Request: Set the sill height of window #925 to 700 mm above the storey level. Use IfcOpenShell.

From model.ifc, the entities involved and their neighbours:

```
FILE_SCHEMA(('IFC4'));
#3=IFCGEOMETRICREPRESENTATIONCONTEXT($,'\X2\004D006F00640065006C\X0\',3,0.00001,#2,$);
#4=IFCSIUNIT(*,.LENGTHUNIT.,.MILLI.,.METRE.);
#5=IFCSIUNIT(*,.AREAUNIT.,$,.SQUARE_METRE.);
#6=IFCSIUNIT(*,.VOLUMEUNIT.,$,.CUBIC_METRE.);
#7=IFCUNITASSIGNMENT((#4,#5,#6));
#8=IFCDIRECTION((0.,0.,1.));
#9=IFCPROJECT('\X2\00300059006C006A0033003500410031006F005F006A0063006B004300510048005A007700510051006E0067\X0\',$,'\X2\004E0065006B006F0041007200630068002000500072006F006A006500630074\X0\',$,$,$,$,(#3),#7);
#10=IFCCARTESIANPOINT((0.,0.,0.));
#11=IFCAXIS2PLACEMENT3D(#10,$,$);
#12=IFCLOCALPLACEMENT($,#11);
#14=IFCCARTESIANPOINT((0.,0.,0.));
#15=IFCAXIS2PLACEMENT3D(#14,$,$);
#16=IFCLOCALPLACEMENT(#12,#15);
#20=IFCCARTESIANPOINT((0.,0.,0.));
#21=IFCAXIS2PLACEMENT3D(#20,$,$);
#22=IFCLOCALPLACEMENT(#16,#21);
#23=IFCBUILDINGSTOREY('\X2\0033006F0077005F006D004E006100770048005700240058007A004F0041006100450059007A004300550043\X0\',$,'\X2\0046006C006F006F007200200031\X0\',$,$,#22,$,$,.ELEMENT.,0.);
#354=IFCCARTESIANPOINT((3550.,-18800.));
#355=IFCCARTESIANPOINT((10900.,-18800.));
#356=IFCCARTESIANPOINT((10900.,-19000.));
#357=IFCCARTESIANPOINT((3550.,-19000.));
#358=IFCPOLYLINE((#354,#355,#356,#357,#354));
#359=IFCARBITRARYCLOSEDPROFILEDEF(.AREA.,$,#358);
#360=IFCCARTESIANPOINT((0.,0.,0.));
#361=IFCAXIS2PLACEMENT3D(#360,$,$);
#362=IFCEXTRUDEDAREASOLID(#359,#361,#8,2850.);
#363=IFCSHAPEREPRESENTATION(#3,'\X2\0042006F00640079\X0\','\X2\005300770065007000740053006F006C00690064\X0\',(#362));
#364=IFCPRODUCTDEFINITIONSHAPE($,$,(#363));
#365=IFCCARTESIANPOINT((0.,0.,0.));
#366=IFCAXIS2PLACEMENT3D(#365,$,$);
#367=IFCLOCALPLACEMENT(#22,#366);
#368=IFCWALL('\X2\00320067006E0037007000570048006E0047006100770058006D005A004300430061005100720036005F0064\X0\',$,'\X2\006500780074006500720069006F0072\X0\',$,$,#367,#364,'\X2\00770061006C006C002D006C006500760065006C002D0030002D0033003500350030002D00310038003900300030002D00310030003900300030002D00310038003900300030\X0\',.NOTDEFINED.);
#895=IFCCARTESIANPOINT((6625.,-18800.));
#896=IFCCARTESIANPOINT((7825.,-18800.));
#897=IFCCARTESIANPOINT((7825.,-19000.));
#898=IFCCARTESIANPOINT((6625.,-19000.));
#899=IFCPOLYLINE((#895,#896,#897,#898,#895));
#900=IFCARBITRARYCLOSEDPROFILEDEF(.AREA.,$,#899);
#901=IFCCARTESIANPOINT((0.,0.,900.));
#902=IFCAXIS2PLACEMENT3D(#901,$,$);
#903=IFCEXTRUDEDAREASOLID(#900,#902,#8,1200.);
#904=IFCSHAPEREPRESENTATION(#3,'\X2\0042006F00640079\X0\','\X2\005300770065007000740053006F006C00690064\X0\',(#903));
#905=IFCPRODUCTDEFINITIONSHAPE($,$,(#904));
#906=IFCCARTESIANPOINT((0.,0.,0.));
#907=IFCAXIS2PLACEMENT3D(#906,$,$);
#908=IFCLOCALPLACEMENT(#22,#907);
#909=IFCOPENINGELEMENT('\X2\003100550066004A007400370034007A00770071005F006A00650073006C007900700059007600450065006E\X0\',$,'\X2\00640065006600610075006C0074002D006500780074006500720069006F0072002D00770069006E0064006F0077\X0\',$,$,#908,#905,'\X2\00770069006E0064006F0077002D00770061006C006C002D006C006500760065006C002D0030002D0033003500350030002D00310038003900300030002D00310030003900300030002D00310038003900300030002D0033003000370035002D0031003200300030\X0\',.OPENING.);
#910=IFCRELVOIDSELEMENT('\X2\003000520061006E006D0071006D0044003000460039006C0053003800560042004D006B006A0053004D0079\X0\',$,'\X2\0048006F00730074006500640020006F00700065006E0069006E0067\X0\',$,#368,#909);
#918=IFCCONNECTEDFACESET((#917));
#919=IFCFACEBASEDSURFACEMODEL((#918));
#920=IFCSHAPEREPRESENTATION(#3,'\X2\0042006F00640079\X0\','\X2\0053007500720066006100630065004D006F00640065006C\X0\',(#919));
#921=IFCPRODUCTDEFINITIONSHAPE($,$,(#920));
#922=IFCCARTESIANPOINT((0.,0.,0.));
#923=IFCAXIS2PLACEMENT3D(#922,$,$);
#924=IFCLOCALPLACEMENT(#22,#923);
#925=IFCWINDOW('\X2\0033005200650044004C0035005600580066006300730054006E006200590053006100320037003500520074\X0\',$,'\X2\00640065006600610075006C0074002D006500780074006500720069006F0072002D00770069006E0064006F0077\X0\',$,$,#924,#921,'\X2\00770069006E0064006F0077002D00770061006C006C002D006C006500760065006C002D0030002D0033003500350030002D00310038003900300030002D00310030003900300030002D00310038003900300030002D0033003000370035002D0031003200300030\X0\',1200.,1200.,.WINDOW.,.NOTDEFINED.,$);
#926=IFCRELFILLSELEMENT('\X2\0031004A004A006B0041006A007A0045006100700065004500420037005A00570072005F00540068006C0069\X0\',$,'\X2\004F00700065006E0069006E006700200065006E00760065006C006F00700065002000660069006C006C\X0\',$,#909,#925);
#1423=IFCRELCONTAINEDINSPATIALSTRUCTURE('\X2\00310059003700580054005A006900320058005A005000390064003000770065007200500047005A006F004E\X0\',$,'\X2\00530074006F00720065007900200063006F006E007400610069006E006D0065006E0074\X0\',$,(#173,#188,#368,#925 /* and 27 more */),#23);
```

```python
import numpy as np
import ifcopenshell
import ifcopenshell.api.geometry
import ifcopenshell.geom
import ifcopenshell.util.element
import ifcopenshell.util.placement
import ifcopenshell.util.shape
import ifcopenshell.util.unit

model = ifcopenshell.open("model.ifc")
unit_scale = ifcopenshell.util.unit.calculate_unit_scale(model)

window = model.by_guid("3ReDL5VXfcsTnbYSa275Rt")
opening = window.FillsVoids[0].RelatingOpeningElement
storey = ifcopenshell.util.element.get_container(window, ifc_class="IfcBuildingStorey")
level = ifcopenshell.util.placement.get_local_placement(storey.ObjectPlacement)[2, 3]

# The opening's origin need not be at the sill, so measure its lowest point.
shape = ifcopenshell.geom.create_shape(ifcopenshell.geom.settings(), opening)
bottom = ifcopenshell.util.shape.get_shape_bottom_elevation(shape, shape.geometry) / unit_scale
dz = level + 700.0 - bottom

shift = np.array([0.0, 0.0, dz])
# The window is not placed relative to its opening, so move both.
for product in (opening, window):
    matrix = ifcopenshell.util.placement.get_local_placement(product.ObjectPlacement)
    matrix[:3, 3] += shift
    ifcopenshell.api.geometry.edit_object_placement(model, product=product, matrix=matrix, is_si=False)

print(f"moved by {dz * unit_scale:+.3f} m")

model.write("model-out.ifc")
```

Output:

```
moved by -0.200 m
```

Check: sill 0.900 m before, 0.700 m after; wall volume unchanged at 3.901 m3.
